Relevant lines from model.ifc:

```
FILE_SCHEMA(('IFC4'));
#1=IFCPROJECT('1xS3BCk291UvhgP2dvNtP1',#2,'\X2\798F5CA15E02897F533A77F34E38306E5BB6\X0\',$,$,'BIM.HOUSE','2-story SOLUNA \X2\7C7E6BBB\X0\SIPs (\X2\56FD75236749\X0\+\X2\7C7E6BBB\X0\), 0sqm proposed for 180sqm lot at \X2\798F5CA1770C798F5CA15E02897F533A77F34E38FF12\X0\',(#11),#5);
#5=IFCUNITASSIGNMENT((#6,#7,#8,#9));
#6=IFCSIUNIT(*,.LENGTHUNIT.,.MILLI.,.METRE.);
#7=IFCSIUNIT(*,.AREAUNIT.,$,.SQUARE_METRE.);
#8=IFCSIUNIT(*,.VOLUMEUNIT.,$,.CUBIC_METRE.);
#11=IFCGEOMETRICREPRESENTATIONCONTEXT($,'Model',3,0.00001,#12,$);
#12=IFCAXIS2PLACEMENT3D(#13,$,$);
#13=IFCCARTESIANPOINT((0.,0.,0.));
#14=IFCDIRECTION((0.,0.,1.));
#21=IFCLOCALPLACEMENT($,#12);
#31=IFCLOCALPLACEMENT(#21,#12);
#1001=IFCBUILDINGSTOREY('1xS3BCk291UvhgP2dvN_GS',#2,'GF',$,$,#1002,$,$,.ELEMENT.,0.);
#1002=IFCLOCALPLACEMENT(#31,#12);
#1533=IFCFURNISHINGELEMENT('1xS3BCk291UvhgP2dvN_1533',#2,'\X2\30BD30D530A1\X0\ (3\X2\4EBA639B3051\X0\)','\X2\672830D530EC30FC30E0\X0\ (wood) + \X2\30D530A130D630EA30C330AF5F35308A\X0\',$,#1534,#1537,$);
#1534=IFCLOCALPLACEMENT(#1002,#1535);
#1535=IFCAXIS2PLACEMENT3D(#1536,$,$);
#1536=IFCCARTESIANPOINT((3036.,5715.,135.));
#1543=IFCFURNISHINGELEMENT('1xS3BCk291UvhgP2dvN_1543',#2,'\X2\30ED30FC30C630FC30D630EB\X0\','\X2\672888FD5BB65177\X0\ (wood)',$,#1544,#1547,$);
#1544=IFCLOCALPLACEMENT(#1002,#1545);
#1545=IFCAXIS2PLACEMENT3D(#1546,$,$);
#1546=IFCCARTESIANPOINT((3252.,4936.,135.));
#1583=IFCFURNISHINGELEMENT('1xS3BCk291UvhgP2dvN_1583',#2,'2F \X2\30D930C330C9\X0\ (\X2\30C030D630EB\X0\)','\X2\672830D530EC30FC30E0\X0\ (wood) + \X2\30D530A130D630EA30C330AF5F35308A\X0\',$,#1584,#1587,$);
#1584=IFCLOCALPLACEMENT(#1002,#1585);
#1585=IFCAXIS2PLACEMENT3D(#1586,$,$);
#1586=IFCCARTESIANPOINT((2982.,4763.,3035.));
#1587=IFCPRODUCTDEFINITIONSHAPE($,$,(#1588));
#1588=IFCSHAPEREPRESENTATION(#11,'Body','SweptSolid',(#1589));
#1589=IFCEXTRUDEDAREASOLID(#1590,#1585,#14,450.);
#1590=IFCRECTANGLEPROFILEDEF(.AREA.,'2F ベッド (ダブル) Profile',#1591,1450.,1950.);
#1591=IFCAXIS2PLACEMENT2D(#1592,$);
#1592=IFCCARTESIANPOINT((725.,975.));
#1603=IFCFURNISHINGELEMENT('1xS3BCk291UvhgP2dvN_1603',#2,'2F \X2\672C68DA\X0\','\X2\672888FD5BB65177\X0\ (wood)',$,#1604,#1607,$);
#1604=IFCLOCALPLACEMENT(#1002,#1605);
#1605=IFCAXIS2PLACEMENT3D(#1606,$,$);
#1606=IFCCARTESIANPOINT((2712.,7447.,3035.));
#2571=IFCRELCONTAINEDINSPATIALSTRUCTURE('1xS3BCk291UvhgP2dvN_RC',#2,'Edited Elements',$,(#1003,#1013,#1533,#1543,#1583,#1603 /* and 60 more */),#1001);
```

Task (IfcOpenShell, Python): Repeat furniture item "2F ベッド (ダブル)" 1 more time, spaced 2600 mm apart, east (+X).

```python
import numpy as np
import ifcopenshell
import ifcopenshell.api.geometry
import ifcopenshell.api.root
import ifcopenshell.util.element
import ifcopenshell.util.placement

model = ifcopenshell.open("model.ifc")


def reuse_history(source, copy):
    """copy_class also copies each property set's owner history, people and application; keep the originals."""
    for rel in copy.IsDefinedBy:
        if rel.is_a("IfcRelDefinesByProperties") and (history := rel.RelatingPropertyDefinition.OwnerHistory):
            rel.RelatingPropertyDefinition.OwnerHistory = source.OwnerHistory
            ifcopenshell.util.element.remove_deep2(model, history)


source = model.by_guid("1xS3BCk291UvhgP2dvN_1583")
base = ifcopenshell.util.placement.get_local_placement(source.ObjectPlacement)
step = np.array([1.0, 0.0, 0.0]) * 2600.0

for i in range(1, 2):
    copy = ifcopenshell.api.root.copy_class(model, product=source)
    copy.Representation = ifcopenshell.util.element.copy_deep(
        model, source.Representation, exclude=["IfcGeometricRepresentationContext", "IfcRepresentationMap"]
    )
    reuse_history(source, copy)
    matrix = base.copy()
    matrix[:3, 3] += i * step
    print("added at", matrix[:3, 3].round(3) + 0.0)
    ifcopenshell.api.geometry.edit_object_placement(model, product=copy, matrix=matrix, is_si=False)

model.write("model_rev.ifc")
```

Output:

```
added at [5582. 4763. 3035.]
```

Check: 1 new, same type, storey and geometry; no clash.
